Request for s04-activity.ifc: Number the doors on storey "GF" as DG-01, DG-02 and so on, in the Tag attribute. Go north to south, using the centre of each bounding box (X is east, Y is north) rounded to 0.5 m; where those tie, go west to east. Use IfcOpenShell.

First a look at what the model holds.

```python
import ifcopenshell
import ifcopenshell.util.element
import ifcopenshell.util.placement

model = ifcopenshell.open("s04-activity.ifc")
print(model.schema)
storey = next(s for s in model.by_type("IfcBuildingStorey") if s.Name == "GF")
doors = [e for e in ifcopenshell.util.element.get_decomposition(storey) if e.is_a("IfcDoor")]
for e in sorted(doors, key=lambda e: e.id()):
    origin = ifcopenshell.util.placement.get_local_placement(e.ObjectPlacement)[:3, 3]
    print(e.id(), e.Tag, e.Name, origin.round(2) + 0.0, sep=" | ")
```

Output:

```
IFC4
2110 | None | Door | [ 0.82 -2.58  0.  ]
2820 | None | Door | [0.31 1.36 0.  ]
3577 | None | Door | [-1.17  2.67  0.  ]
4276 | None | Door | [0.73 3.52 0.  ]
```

```python
import ifcopenshell
import ifcopenshell.geom
import ifcopenshell.util.element
import ifcopenshell.util.shape

model = ifcopenshell.open("s04-activity.ifc")
settings = ifcopenshell.geom.settings()
settings.set("use-world-coords", True)


def centre(element):
    shape = ifcopenshell.geom.create_shape(settings, element)
    return ifcopenshell.util.shape.get_bbox_centroid(shape.geometry)


storey = next(s for s in model.by_type("IfcBuildingStorey") if s.Name == "GF")
doors = [e for e in ifcopenshell.util.element.get_decomposition(storey) if e.is_a("IfcDoor")]

# Insertion points can sit at a corner or the storey origin, so sort by the geometry (in metres).
centres = {e: centre(e) for e in doors}
doors.sort(key=lambda e: (-round(centres[e][1] / 0.5), centres[e][0]))

for i, e in enumerate(doors, start=1):
    number = f"DG-{i:02d}"
    e.Tag = number
    print(e.id(), number)

model.write("s04-activity_rev.ifc")
```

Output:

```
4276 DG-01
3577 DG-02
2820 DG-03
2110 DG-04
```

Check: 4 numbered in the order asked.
